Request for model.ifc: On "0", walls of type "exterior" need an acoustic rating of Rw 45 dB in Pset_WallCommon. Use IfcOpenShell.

First a look at what the model holds.

```python
import ifcopenshell
import ifcopenshell.util.element

model = ifcopenshell.open("model.ifc")
print(model.schema)
storey = next(s for s in model.by_type("IfcBuildingStorey") if s.Name == "0")
walls = [e for e in ifcopenshell.util.element.get_decomposition(storey) if e.is_a("IfcWall")]
seen = {}
for e in walls:
    element_type = ifcopenshell.util.element.get_type(e)
    key = (element_type.Name if element_type != e and element_type else None, ifcopenshell.util.element.get_pset(e, "Pset_WallCommon", "AcousticRating"))
    seen[key] = seen.get(key, 0) + 1
for (name, value), count in sorted(seen.items(), key=str):
    print(count, "x", name, "|", value)
```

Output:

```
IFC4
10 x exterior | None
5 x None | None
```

```python
import ifcopenshell
import ifcopenshell.api.pset
import ifcopenshell.util.element

model = ifcopenshell.open("model.ifc")

storey = next(s for s in model.by_type("IfcBuildingStorey") if s.Name == "0")
walls = [e for e in ifcopenshell.util.element.get_decomposition(storey) if e.is_a("IfcWall")]

count = 0
for e in walls:
    element_type = ifcopenshell.util.element.get_type(e)
    if element_type in (None, e) or element_type.Name != "exterior":
        continue
    # add_pset returns the element's existing set when there is one.
    pset = ifcopenshell.api.pset.add_pset(model, product=e, name="Pset_WallCommon")
    ifcopenshell.api.pset.edit_pset(model, pset=pset, properties={"AcousticRating": "Rw 45 dB"})
    count += 1

print(count, "walls updated")

model.write("model_rev.ifc")
```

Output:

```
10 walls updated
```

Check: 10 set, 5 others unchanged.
